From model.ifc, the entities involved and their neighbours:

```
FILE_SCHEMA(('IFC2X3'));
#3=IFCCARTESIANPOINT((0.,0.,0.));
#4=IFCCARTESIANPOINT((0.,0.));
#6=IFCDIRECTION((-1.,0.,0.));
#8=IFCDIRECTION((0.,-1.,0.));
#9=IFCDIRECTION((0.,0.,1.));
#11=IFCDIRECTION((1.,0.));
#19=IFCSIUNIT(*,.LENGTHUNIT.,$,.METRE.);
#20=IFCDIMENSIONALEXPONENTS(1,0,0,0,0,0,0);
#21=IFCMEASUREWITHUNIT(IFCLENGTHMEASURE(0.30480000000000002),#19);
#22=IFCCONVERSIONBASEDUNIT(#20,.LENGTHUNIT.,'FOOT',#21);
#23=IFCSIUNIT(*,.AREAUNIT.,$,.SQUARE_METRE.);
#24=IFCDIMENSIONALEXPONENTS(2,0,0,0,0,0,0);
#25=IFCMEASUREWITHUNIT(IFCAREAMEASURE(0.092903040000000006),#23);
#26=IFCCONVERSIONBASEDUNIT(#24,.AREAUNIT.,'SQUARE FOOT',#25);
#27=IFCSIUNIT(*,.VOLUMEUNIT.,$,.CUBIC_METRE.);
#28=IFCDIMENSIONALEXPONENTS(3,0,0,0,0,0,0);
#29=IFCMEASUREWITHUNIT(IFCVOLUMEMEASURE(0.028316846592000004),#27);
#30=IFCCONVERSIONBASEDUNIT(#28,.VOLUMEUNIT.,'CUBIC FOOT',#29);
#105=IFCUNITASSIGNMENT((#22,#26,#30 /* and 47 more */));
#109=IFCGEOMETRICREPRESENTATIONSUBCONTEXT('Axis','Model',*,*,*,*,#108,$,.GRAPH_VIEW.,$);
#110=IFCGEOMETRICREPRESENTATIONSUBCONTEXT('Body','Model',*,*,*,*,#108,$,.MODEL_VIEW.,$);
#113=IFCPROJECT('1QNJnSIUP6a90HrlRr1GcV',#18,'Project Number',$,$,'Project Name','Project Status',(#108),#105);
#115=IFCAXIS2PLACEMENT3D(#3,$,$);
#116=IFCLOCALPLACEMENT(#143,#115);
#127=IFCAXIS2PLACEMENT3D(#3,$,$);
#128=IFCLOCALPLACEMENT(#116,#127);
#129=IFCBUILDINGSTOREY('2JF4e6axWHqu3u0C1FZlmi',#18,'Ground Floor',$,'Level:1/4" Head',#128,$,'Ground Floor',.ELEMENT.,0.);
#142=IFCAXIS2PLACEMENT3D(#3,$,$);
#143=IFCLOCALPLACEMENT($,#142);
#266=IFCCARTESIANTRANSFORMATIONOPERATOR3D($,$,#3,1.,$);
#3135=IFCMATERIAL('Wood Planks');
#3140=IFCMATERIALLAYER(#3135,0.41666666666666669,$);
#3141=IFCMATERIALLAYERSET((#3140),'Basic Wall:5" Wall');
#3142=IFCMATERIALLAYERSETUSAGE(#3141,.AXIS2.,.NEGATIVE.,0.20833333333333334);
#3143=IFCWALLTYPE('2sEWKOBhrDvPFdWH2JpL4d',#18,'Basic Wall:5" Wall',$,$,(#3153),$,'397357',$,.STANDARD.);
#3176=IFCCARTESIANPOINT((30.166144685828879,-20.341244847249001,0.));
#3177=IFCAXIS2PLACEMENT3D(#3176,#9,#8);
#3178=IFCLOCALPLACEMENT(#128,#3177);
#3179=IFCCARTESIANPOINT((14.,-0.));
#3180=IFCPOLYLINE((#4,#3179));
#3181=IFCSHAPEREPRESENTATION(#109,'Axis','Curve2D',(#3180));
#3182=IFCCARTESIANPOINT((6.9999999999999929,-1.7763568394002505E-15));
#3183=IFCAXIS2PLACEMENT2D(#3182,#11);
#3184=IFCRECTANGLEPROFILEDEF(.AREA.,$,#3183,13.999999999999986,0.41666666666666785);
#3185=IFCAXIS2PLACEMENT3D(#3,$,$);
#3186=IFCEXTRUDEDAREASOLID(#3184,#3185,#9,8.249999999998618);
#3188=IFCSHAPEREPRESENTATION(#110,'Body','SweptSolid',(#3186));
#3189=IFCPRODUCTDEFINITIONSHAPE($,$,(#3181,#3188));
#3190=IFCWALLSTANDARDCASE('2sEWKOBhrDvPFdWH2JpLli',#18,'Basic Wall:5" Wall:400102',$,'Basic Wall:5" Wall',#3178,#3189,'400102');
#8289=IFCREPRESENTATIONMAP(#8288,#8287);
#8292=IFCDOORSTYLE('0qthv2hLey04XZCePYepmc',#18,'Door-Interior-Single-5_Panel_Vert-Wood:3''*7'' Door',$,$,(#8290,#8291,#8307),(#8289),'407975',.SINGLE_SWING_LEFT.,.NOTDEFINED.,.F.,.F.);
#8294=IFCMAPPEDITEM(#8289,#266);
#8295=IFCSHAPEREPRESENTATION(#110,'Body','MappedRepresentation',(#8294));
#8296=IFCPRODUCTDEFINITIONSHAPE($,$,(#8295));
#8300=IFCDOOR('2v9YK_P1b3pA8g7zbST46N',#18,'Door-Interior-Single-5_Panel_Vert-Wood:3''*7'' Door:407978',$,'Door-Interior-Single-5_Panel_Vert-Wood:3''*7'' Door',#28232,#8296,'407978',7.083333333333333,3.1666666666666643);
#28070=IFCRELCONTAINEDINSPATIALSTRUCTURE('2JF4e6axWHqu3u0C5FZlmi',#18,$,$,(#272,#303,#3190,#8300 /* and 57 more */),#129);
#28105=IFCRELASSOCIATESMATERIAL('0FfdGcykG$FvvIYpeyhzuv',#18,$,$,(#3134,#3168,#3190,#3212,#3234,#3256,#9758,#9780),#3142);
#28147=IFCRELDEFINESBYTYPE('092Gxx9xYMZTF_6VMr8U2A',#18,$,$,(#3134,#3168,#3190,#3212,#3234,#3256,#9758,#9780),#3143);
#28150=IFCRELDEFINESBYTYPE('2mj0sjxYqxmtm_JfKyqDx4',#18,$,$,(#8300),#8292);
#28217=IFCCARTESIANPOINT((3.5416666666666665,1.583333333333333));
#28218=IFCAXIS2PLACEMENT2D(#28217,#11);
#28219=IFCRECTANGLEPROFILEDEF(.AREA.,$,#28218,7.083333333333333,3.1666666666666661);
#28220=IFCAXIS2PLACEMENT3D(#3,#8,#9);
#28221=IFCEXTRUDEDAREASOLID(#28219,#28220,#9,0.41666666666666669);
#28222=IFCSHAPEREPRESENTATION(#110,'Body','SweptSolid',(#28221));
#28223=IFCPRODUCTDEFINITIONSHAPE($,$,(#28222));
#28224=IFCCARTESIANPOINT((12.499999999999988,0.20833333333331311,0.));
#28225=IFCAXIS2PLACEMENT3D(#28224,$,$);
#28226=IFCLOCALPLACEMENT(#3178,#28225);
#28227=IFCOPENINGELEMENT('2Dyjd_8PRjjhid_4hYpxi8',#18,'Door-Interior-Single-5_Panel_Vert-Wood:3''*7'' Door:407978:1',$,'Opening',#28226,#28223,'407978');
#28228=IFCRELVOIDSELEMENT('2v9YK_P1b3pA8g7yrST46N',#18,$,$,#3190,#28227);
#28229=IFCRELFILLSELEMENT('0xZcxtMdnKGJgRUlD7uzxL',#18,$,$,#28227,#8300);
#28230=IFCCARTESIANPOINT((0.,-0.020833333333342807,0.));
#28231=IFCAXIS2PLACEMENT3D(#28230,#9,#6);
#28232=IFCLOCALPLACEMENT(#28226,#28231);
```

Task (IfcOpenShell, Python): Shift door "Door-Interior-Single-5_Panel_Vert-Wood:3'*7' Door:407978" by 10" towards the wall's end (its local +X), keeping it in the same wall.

```python
import ifcopenshell
import ifcopenshell.api.geometry
import ifcopenshell.util.placement
import ifcopenshell.util.unit

model = ifcopenshell.open("model.ifc")
unit_scale = ifcopenshell.util.unit.calculate_unit_scale(model)

door = model.by_guid("2v9YK_P1b3pA8g7zbST46N")
opening = door.FillsVoids[0].RelatingOpeningElement
wall = opening.VoidsElements[0].RelatingBuildingElement

wall_matrix = ifcopenshell.util.placement.get_local_placement(wall.ObjectPlacement)
shift = wall_matrix[:3, 0] * 10 * 0.0254 / unit_scale
before = ifcopenshell.util.placement.get_local_placement(door.ObjectPlacement)[:3, 3].copy()

# The door is placed relative to its opening, so it follows when the opening moves.
matrix = ifcopenshell.util.placement.get_local_placement(opening.ObjectPlacement)
matrix[:3, 3] += shift
ifcopenshell.api.geometry.edit_object_placement(
    model, product=opening, matrix=matrix, is_si=False, should_transform_children=True
)

after = ifcopenshell.util.placement.get_local_placement(door.ObjectPlacement)[:3, 3]
print("door moved by", (after - before).round(3) + 0.0)

model.write("model_rev.ifc")
```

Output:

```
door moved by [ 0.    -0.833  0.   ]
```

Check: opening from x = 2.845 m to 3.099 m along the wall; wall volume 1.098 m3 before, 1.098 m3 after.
